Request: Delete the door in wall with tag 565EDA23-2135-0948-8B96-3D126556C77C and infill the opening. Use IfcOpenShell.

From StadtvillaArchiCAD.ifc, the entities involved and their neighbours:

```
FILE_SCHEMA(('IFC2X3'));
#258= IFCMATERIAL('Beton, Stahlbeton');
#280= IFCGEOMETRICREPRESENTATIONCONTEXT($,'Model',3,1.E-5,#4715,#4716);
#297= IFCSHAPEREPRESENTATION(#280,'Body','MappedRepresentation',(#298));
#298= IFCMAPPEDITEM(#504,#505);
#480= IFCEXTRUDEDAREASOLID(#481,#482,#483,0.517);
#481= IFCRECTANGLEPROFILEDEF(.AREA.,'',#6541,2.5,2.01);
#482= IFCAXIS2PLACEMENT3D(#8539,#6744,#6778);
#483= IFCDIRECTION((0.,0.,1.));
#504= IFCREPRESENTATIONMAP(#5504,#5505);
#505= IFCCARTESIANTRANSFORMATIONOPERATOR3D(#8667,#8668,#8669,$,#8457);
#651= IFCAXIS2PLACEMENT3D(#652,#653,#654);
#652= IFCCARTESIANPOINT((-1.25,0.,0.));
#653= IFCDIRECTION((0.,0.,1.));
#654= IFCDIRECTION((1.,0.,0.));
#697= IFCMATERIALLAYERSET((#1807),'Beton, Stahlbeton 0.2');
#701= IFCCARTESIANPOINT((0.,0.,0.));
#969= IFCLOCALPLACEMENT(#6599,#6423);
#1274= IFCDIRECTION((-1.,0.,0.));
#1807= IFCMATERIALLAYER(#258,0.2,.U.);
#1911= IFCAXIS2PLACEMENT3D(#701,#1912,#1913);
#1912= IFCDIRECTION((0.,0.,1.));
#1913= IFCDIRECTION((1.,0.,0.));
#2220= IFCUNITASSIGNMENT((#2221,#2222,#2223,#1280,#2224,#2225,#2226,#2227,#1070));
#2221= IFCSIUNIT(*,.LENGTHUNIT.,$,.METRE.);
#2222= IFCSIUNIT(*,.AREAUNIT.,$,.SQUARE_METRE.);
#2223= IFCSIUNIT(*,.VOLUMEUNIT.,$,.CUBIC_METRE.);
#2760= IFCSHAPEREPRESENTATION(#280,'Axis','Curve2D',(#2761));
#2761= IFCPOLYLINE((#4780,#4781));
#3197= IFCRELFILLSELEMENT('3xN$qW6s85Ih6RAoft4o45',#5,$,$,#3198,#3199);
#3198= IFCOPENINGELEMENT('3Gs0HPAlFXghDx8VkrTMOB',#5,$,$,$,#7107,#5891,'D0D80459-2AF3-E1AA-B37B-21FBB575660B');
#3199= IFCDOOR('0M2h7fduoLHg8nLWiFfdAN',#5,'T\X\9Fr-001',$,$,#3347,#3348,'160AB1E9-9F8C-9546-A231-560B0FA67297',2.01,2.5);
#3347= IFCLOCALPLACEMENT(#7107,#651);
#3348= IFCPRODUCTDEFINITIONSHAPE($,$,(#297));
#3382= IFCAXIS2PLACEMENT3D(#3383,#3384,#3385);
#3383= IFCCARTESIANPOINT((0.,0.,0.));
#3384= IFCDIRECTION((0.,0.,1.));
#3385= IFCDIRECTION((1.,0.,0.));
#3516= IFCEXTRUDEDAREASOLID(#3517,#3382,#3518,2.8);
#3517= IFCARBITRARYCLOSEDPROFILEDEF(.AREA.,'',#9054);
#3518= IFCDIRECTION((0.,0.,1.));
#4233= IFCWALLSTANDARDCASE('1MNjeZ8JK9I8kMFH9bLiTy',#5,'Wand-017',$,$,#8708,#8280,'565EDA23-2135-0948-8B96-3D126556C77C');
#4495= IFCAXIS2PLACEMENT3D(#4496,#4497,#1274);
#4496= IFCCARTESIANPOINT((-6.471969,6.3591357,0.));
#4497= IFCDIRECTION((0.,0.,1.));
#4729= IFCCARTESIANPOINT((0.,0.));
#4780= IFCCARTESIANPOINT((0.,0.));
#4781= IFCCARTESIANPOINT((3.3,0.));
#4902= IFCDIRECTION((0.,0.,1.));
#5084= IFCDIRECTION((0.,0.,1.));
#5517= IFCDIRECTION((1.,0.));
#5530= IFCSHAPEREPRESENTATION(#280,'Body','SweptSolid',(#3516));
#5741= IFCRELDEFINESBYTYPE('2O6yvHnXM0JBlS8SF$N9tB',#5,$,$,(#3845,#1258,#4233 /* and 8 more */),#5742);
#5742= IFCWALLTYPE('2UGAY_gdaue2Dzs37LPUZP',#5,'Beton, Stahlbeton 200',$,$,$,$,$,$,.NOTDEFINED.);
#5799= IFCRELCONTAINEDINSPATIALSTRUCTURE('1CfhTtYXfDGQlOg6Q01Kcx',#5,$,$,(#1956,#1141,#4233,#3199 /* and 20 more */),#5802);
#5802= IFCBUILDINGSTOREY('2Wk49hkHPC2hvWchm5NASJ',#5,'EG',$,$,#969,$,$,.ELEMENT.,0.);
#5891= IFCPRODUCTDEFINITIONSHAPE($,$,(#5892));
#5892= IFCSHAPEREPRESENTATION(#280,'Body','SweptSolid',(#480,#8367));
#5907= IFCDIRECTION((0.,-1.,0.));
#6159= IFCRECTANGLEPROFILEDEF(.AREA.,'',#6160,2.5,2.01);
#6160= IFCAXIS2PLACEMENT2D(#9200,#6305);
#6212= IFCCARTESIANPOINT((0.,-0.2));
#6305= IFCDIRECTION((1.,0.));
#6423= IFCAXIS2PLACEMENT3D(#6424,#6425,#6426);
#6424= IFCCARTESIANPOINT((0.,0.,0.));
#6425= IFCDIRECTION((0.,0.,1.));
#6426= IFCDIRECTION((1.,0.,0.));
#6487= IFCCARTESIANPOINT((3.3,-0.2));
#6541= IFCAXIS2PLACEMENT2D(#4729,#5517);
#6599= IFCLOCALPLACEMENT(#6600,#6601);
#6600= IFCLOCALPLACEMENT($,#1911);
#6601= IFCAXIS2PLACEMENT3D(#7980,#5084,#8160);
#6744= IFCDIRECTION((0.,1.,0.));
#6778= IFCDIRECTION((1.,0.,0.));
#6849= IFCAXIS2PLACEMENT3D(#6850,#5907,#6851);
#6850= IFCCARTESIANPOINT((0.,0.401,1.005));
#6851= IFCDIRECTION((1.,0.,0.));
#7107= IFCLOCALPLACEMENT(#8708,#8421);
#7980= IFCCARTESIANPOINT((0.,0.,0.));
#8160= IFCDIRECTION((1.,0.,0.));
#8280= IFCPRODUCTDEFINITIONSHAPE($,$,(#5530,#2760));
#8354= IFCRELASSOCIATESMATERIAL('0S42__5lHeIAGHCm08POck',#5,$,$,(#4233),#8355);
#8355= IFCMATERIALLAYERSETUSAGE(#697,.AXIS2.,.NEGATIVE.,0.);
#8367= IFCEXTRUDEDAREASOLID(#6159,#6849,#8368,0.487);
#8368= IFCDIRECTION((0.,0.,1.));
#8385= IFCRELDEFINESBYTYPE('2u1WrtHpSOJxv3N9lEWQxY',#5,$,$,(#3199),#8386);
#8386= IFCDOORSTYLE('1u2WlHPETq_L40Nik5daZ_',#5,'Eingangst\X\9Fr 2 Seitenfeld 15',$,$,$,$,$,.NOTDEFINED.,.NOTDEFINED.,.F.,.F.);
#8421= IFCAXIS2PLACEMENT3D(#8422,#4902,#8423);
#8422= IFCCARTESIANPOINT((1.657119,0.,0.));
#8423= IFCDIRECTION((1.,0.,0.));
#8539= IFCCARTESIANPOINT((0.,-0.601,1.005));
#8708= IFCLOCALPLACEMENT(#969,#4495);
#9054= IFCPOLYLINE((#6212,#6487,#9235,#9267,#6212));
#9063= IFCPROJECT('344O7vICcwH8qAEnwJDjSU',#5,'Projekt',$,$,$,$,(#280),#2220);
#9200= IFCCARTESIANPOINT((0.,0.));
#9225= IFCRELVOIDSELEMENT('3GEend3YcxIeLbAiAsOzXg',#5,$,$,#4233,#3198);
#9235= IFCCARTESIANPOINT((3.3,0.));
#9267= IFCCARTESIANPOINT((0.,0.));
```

```python
import ifcopenshell
import ifcopenshell.api.feature
import ifcopenshell.api.root
import ifcopenshell.geom
import ifcopenshell.util.shape

model = ifcopenshell.open("StadtvillaArchiCAD.ifc")
settings = ifcopenshell.geom.settings()


def volume(element):
    """Net volume in cubic metres, openings subtracted."""
    shape = ifcopenshell.geom.create_shape(settings, element)
    return ifcopenshell.util.shape.get_volume(shape.geometry)


door = model.by_guid("0M2h7fduoLHg8nLWiFfdAN")
opening = door.FillsVoids[0].RelatingOpeningElement
wall = opening.VoidsElements[0].RelatingBuildingElement
before = volume(wall)

ifcopenshell.api.root.remove_product(model, product=door)
ifcopenshell.api.feature.remove_feature(model, feature=opening)

after = volume(wall)

print(f"wall volume {before:.3f} -> {after:.3f} m3")

model.write("StadtvillaArchiCAD_edited.ifc")
```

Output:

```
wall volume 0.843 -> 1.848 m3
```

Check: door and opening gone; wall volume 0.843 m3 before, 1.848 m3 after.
